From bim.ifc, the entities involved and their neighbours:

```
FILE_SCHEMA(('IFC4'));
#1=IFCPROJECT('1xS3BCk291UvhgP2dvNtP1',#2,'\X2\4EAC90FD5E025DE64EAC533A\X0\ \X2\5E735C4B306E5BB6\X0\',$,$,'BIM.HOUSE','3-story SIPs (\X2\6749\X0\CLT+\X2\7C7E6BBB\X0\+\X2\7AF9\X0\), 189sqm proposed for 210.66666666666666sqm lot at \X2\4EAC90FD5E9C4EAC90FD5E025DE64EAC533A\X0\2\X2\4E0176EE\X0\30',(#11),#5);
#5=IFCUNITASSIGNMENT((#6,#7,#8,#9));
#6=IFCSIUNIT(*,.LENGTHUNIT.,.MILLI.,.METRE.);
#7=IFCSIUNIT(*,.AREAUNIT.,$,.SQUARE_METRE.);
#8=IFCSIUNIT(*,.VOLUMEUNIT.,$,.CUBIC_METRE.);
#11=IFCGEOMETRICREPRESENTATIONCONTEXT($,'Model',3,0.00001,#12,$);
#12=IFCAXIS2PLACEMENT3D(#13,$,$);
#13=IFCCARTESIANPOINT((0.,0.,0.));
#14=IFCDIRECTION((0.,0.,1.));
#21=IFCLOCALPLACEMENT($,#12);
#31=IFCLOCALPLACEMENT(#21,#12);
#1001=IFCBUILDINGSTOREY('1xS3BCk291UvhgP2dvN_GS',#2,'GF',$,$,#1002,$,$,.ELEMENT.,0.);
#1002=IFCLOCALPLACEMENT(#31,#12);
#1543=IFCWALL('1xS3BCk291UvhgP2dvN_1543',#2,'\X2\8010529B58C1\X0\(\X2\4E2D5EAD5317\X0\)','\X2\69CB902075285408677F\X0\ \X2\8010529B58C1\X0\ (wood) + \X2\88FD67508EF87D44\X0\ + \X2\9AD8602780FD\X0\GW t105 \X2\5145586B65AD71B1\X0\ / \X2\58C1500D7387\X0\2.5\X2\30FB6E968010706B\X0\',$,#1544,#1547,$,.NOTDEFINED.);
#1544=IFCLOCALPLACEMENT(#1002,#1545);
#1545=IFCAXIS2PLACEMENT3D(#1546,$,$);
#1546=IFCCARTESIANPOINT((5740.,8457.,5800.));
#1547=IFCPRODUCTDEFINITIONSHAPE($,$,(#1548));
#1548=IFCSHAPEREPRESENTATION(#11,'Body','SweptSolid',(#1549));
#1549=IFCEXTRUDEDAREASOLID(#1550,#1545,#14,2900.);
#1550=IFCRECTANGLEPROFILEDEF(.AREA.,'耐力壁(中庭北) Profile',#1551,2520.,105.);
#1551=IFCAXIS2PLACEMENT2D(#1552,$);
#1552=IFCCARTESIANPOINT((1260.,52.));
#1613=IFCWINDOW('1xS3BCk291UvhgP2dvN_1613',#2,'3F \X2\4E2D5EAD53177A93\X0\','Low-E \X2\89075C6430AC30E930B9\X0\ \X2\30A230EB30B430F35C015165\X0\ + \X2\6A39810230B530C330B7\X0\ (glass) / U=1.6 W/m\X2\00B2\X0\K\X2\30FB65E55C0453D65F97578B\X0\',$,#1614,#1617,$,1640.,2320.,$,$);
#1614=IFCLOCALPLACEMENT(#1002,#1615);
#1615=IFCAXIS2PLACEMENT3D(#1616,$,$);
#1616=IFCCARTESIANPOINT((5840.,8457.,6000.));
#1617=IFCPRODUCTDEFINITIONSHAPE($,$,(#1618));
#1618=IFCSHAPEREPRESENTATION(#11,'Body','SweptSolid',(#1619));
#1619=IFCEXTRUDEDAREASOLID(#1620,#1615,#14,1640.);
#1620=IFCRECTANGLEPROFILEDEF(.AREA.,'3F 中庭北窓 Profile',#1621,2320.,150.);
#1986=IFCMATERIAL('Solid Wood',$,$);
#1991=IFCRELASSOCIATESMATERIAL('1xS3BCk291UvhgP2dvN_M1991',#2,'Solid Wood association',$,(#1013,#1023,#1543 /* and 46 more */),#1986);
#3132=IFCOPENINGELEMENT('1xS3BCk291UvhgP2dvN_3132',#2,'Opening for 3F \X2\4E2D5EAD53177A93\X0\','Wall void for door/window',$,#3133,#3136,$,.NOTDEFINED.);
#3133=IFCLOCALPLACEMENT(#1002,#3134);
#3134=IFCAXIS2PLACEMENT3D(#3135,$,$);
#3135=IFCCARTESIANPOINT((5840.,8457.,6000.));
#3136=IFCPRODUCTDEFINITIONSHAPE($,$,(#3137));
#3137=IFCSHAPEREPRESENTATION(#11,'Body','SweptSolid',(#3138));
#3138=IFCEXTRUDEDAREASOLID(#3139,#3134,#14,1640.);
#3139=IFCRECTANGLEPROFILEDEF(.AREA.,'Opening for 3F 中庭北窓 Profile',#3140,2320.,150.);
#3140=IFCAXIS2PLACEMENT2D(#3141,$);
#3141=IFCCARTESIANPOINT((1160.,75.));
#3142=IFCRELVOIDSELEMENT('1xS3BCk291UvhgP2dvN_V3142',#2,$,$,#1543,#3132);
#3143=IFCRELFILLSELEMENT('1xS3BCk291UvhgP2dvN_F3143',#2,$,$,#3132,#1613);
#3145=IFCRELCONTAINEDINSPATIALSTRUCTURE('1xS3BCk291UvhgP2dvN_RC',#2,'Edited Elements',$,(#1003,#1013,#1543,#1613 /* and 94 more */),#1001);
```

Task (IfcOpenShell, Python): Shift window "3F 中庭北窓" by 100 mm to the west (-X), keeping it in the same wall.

```python
import ifcopenshell
import ifcopenshell.api.geometry
import ifcopenshell.util.placement
import ifcopenshell.util.unit

model = ifcopenshell.open("bim.ifc")
unit_scale = ifcopenshell.util.unit.calculate_unit_scale(model)

window = model.by_guid("1xS3BCk291UvhgP2dvN_1613")
opening = window.FillsVoids[0].RelatingOpeningElement
wall = opening.VoidsElements[0].RelatingBuildingElement

wall_matrix = ifcopenshell.util.placement.get_local_placement(wall.ObjectPlacement)
shift = wall_matrix[:3, 0] * -0.1 / unit_scale
before = ifcopenshell.util.placement.get_local_placement(window.ObjectPlacement)[:3, 3].copy()

# The window is not placed relative to its opening, so move both.
for product in (opening, window):
    matrix = ifcopenshell.util.placement.get_local_placement(product.ObjectPlacement)
    matrix[:3, 3] += shift
    ifcopenshell.api.geometry.edit_object_placement(model, product=product, matrix=matrix, is_si=False)

after = ifcopenshell.util.placement.get_local_placement(window.ObjectPlacement)[:3, 3]
print("window moved by", (after - before).round(3) + 0.0)

model.write("bim_rev.ifc")
```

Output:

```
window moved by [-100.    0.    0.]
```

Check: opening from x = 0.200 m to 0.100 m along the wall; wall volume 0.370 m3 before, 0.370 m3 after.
